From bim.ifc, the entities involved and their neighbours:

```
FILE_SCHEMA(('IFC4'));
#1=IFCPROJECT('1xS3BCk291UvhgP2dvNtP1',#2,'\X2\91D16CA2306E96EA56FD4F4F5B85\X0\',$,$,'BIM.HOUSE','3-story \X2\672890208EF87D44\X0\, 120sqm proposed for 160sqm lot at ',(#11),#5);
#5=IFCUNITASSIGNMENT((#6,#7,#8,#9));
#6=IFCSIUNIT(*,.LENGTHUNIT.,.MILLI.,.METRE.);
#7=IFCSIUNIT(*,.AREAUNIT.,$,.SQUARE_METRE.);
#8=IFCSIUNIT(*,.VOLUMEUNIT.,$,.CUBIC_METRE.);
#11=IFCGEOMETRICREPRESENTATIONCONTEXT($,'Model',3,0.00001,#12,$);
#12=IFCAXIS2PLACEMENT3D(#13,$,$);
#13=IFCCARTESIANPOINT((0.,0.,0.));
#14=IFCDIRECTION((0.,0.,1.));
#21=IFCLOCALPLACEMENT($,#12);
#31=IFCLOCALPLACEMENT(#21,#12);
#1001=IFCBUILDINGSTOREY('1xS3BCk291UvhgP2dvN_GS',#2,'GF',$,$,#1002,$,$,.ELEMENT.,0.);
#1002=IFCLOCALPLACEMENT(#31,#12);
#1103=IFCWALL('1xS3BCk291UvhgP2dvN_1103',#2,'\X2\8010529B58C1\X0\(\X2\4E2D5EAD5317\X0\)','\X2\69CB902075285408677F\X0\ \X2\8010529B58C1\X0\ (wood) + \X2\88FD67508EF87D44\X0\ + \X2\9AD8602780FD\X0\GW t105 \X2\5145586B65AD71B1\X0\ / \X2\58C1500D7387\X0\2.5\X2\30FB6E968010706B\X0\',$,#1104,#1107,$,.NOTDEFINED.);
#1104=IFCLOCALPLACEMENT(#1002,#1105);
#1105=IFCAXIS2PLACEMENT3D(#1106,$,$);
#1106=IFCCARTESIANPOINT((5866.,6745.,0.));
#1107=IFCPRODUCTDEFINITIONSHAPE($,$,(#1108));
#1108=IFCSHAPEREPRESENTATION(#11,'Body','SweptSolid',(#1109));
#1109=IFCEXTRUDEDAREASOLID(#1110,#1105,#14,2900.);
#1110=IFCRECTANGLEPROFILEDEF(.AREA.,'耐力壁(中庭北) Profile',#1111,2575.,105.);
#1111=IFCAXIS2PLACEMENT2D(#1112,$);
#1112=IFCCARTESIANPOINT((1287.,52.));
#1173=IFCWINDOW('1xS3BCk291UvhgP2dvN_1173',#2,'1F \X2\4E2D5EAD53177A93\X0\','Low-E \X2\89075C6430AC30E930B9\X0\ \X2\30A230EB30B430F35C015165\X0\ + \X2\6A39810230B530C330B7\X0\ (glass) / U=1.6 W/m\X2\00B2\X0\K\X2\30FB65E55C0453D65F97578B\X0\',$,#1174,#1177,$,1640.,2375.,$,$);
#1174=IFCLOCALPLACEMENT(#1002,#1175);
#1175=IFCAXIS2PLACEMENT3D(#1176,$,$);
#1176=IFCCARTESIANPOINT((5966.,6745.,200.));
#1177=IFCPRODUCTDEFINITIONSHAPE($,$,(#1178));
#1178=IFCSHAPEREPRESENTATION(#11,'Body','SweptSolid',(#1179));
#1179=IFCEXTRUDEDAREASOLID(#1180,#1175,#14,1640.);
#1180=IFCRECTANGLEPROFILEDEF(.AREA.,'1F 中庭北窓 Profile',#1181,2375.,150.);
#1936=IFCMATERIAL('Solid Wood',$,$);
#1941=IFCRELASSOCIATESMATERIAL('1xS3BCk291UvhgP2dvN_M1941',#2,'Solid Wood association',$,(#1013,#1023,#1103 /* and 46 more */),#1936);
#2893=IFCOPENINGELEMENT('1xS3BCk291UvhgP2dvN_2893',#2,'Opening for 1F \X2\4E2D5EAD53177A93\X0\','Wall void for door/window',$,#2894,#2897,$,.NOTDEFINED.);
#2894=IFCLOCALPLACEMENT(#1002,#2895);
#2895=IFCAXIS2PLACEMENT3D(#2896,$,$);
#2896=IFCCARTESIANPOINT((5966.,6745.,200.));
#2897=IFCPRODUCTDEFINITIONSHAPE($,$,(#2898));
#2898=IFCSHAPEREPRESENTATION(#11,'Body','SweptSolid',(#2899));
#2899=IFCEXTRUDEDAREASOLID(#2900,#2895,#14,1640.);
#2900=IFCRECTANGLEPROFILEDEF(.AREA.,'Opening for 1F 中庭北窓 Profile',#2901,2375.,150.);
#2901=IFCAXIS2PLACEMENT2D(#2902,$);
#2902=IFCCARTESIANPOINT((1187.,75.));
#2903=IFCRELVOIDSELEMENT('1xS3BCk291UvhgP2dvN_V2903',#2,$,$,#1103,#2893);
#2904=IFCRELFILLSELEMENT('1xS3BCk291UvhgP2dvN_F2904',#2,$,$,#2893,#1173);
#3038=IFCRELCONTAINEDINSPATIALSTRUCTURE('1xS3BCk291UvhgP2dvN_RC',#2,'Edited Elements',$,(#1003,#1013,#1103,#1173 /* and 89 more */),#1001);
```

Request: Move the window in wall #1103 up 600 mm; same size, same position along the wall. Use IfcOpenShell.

```python
import numpy as np
import ifcopenshell
import ifcopenshell.api.geometry
import ifcopenshell.util.placement
import ifcopenshell.util.unit

model = ifcopenshell.open("bim.ifc")
unit_scale = ifcopenshell.util.unit.calculate_unit_scale(model)

window = model.by_id(1173)
opening = window.FillsVoids[0].RelatingOpeningElement
dz = 600.0

shift = np.array([0.0, 0.0, dz])
# The window is not placed relative to its opening, so move both.
for product in (opening, window):
    matrix = ifcopenshell.util.placement.get_local_placement(product.ObjectPlacement)
    matrix[:3, 3] += shift
    ifcopenshell.api.geometry.edit_object_placement(model, product=product, matrix=matrix, is_si=False)

print(f"moved by {dz * unit_scale:+.3f} m")

model.write("bim_updated.ifc")
```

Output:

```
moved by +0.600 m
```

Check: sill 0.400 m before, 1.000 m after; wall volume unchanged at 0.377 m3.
